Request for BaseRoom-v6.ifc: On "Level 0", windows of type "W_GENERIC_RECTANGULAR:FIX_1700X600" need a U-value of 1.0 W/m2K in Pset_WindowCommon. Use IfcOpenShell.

First a look at what the model holds.

```python
import ifcopenshell
import ifcopenshell.util.element

model = ifcopenshell.open("BaseRoom-v6.ifc")
print(model.schema)
storey = next(s for s in model.by_type("IfcBuildingStorey") if s.Name == "Level 0")
windows = [e for e in ifcopenshell.util.element.get_decomposition(storey) if e.is_a("IfcWindow")]
seen = {}
for e in windows:
    element_type = ifcopenshell.util.element.get_type(e)
    key = (element_type.Name if element_type != e and element_type else None, ifcopenshell.util.element.get_pset(e, "Pset_WindowCommon", "ThermalTransmittance"))
    seen[key] = seen.get(key, 0) + 1
for (name, value), count in sorted(seen.items(), key=str):
    print(count, "x", name, "|", value)
```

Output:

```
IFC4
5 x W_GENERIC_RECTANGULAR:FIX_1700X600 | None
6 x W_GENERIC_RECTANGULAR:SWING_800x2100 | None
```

```python
import ifcopenshell
import ifcopenshell.api.pset
import ifcopenshell.util.element

model = ifcopenshell.open("BaseRoom-v6.ifc")

storey = next(s for s in model.by_type("IfcBuildingStorey") if s.Name == "Level 0")
windows = [e for e in ifcopenshell.util.element.get_decomposition(storey) if e.is_a("IfcWindow")]

count = 0
for e in windows:
    element_type = ifcopenshell.util.element.get_type(e)
    if element_type in (None, e) or element_type.Name != "W_GENERIC_RECTANGULAR:FIX_1700X600":
        continue
    # add_pset returns the element's existing set when there is one.
    pset = ifcopenshell.api.pset.add_pset(model, product=e, name="Pset_WindowCommon")
    ifcopenshell.api.pset.edit_pset(model, pset=pset, properties={"ThermalTransmittance": 1.0})
    count += 1

print(count, "windows updated")

model.write("BaseRoom-v6_updated.ifc")
```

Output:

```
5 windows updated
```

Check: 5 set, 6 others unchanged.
